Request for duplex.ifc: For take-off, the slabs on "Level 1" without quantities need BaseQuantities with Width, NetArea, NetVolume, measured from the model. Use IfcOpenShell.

First a look at what the model holds.

```python
import ifcopenshell
import ifcopenshell.util.element
import ifcopenshell.util.unit

model = ifcopenshell.open("duplex.ifc")
print(model.schema)
for unit_type in ("LENGTHUNIT", "AREAUNIT", "VOLUMEUNIT"):
    print(unit_type, ifcopenshell.util.unit.calculate_unit_scale(model, unit_type))
storey = next(s for s in model.by_type("IfcBuildingStorey") if s.Name == "Level 1")
slabs = [e for e in ifcopenshell.util.element.get_decomposition(storey) if e.is_a("IfcSlab")]
for e in sorted(slabs, key=lambda e: e.id()):
    print(e.id(), e.is_a(), e.Name, list(ifcopenshell.util.element.get_psets(e, qtos_only=True)), sep=" | ")
```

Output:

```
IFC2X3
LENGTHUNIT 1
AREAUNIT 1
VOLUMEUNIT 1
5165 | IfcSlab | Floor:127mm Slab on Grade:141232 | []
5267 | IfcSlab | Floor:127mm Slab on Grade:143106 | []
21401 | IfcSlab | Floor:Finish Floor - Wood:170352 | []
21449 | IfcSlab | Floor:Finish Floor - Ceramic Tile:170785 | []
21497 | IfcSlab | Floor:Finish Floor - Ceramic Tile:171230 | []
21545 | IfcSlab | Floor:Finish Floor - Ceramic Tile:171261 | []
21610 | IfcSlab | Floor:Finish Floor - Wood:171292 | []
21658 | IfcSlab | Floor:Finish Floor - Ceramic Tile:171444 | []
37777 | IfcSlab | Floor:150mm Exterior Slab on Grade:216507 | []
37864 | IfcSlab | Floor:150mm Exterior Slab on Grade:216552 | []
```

```python
import ifcopenshell
import ifcopenshell.api.pset
import ifcopenshell.geom
import ifcopenshell.util.element
import ifcopenshell.util.shape
import ifcopenshell.util.unit

model = ifcopenshell.open("duplex.ifc")
unit_scale = ifcopenshell.util.unit.calculate_unit_scale(model)
area_scale = ifcopenshell.util.unit.calculate_unit_scale(model, "AREAUNIT")
volume_scale = ifcopenshell.util.unit.calculate_unit_scale(model, "VOLUMEUNIT")
settings = ifcopenshell.geom.settings()

storey = next(s for s in model.by_type("IfcBuildingStorey") if s.Name == "Level 1")
slabs = [e for e in ifcopenshell.util.element.get_decomposition(storey) if e.is_a("IfcSlab")]

for e in sorted(slabs, key=lambda e: e.id()):
    if ifcopenshell.util.element.get_psets(e, qtos_only=True, should_inherit=False):
        continue
    # Geometry comes back in metres, in the element's own axes.
    shape = ifcopenshell.geom.create_shape(settings, e)
    values = {
        "Width": ifcopenshell.util.shape.get_z(shape.geometry) / unit_scale,
        "NetArea": ifcopenshell.util.shape.get_footprint_area(shape.geometry) / area_scale,
        "NetVolume": ifcopenshell.util.shape.get_volume(shape.geometry) / volume_scale,
    }
    qto = ifcopenshell.api.pset.add_qto(model, product=e, name="BaseQuantities")
    ifcopenshell.api.pset.edit_qto(model, qto=qto, properties=values)
    print(e.id(), {k: round(v, 3) for k, v in values.items()})

model.write("duplex_rev.ifc")
```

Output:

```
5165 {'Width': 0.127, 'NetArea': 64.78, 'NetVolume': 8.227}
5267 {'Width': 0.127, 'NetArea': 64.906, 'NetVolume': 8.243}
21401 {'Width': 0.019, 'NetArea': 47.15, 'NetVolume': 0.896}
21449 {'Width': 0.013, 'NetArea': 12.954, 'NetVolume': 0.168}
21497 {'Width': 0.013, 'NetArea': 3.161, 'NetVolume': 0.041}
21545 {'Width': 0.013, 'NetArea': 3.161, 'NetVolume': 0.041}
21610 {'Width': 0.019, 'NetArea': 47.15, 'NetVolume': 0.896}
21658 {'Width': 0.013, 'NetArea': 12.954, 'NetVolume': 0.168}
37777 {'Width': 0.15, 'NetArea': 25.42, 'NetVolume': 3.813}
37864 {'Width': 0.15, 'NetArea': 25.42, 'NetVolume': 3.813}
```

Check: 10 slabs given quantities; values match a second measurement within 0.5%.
